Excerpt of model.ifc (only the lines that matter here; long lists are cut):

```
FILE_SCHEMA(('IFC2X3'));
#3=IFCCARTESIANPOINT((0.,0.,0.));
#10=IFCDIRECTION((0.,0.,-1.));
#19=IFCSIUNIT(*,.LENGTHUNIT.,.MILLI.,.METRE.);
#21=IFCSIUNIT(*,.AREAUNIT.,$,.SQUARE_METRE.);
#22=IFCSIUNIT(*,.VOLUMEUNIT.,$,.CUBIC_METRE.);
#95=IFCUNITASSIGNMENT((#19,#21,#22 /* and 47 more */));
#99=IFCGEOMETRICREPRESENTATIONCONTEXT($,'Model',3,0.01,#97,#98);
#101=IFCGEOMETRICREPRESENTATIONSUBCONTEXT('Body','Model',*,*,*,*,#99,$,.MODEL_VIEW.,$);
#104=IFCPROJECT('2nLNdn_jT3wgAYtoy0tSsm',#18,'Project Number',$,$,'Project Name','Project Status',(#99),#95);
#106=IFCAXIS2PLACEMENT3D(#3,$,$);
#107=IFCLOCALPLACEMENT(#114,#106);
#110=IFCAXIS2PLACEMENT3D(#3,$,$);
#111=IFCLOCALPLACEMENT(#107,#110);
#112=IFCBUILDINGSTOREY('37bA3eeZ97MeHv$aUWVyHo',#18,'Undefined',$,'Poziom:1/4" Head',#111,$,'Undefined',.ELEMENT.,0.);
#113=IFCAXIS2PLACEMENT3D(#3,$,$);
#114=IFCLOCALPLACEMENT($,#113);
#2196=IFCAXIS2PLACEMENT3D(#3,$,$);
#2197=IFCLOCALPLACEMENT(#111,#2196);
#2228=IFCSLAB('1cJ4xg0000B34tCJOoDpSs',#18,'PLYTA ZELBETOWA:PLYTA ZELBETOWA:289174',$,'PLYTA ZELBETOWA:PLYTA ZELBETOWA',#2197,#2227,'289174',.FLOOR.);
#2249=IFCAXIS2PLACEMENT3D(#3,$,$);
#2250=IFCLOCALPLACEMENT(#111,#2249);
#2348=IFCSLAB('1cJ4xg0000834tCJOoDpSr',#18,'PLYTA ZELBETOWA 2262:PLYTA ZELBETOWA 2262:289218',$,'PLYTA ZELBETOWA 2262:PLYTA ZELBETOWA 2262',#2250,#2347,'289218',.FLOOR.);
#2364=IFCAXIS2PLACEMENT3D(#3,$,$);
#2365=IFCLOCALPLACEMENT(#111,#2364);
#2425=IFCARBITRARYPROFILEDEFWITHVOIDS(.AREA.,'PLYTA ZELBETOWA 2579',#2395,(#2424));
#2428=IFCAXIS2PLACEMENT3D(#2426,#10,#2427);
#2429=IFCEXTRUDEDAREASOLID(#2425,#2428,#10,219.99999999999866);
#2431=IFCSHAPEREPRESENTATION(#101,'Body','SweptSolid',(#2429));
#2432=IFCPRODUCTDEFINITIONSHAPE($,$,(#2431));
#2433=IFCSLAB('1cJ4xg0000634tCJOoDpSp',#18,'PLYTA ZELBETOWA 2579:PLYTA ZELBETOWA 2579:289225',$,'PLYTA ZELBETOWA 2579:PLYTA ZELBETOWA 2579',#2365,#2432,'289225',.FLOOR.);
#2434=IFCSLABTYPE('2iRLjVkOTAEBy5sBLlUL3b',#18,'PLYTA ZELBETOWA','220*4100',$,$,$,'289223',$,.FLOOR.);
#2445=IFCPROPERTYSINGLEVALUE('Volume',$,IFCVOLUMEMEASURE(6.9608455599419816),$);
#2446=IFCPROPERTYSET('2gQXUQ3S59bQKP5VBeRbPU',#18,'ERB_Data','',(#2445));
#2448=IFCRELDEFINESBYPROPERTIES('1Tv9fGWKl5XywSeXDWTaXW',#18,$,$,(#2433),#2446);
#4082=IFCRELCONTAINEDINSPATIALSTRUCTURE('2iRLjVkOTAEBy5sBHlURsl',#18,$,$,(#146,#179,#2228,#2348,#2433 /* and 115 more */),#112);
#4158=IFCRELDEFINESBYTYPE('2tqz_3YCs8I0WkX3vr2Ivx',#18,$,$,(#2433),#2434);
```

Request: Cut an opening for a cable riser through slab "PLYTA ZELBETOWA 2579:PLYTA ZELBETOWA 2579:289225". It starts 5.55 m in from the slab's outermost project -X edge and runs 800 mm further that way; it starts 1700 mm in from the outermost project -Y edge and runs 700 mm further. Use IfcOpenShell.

```python
import numpy as np
import ifcopenshell
import ifcopenshell.api.feature
import ifcopenshell.api.geometry
import ifcopenshell.api.pset
import ifcopenshell.api.root
import ifcopenshell.geom
import ifcopenshell.util.element
import ifcopenshell.util.placement
import ifcopenshell.util.representation
import ifcopenshell.util.shape
import ifcopenshell.util.unit

model = ifcopenshell.open("model.ifc")
unit_scale = ifcopenshell.util.unit.calculate_unit_scale(model)
volume_scale = ifcopenshell.util.unit.calculate_unit_scale(model, "VOLUMEUNIT")
settings = ifcopenshell.geom.settings()


def volume(element):
    """Net volume in cubic metres, openings subtracted."""
    shape = ifcopenshell.geom.create_shape(settings, element)
    return ifcopenshell.util.shape.get_volume(shape.geometry)


slab = model.by_guid("1cJ4xg0000634tCJOoDpSp")
before = volume(slab)

# Extent in the slab's own axes, in metres. The edges named are its -X and -Y sides.
slab_shape = ifcopenshell.geom.create_shape(settings, slab)
vertices = ifcopenshell.util.shape.get_vertices(slab_shape.geometry)
x_min, y_min, bottom = vertices.min(axis=0)
top = vertices[:, 2].max()

opening = ifcopenshell.api.root.create_entity(model, ifc_class="IfcOpeningElement", name="Cable riser opening")
context = ifcopenshell.util.representation.get_context(model, "Model", "Body", "MODEL_VIEW")
width, depth = 0.8, 0.7
outline = [(0.0, 0.0), (width, 0.0), (width, depth), (0.0, depth), (0.0, 0.0)]
# Overshoot both faces by 50 mm so the cut is clean.
shape = ifcopenshell.api.geometry.add_slab_representation(
    model, context=context, depth=top - bottom + 0.1, polyline=outline
)
ifcopenshell.api.geometry.assign_representation(model, product=opening, representation=shape)

matrix = ifcopenshell.util.placement.get_local_placement(slab.ObjectPlacement)
matrix[:, 3] = matrix @ np.append(np.array([x_min + 5.55, y_min + 1.7, bottom - 0.05]) / unit_scale, 1.0)
ifcopenshell.api.geometry.edit_object_placement(model, product=opening, matrix=matrix, is_si=False)
ifcopenshell.api.feature.add_feature(model, feature=opening, element=slab)

after = volume(slab)

# Update the slab's stored quantities.
pset = model.by_id(ifcopenshell.util.element.get_pset(slab, "ERB_Data", should_inherit=False)["id"])
ifcopenshell.api.pset.edit_pset(model, pset=pset, properties={
    "Volume": model.create_entity("IfcVolumeMeasure", after / volume_scale),
})

print(f"slab volume {before:.3f} -> {after:.3f} m3")

model.write("model_updated.ifc")
```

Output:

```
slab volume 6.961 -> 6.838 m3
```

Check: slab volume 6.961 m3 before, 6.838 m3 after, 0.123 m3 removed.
